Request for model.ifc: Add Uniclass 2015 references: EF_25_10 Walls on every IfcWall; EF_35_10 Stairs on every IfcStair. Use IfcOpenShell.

First a look at what the model holds.

```python
import ifcopenshell

model = ifcopenshell.open("model.ifc")
print(model.schema)
print("classifications:", [c.Name for c in model.by_type("IfcClassification")])
for ifc_class in ("IfcDoor", "IfcRoof", "IfcStair", "IfcWall", "IfcWindow"):
    print(ifc_class, len(model.by_type(ifc_class)))
```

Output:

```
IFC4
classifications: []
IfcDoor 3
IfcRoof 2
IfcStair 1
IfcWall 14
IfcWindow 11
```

```python
import ifcopenshell
import ifcopenshell.api.classification

model = ifcopenshell.open("model.ifc")

system = ifcopenshell.api.classification.add_classification(model, classification="Uniclass 2015")

codes = {
    "IfcWall": ("EF_25_10", "Walls"),
    "IfcStair": ("EF_35_10", "Stairs"),
}
for ifc_class, (code, name) in codes.items():
    products = model.by_type(ifc_class)
    ifcopenshell.api.classification.add_reference(
        model, products=products, classification=system, identification=code, name=name
    )
    print(code, len(products))

model.write("model-out.ifc")
```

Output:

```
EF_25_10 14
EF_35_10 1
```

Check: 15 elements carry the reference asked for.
